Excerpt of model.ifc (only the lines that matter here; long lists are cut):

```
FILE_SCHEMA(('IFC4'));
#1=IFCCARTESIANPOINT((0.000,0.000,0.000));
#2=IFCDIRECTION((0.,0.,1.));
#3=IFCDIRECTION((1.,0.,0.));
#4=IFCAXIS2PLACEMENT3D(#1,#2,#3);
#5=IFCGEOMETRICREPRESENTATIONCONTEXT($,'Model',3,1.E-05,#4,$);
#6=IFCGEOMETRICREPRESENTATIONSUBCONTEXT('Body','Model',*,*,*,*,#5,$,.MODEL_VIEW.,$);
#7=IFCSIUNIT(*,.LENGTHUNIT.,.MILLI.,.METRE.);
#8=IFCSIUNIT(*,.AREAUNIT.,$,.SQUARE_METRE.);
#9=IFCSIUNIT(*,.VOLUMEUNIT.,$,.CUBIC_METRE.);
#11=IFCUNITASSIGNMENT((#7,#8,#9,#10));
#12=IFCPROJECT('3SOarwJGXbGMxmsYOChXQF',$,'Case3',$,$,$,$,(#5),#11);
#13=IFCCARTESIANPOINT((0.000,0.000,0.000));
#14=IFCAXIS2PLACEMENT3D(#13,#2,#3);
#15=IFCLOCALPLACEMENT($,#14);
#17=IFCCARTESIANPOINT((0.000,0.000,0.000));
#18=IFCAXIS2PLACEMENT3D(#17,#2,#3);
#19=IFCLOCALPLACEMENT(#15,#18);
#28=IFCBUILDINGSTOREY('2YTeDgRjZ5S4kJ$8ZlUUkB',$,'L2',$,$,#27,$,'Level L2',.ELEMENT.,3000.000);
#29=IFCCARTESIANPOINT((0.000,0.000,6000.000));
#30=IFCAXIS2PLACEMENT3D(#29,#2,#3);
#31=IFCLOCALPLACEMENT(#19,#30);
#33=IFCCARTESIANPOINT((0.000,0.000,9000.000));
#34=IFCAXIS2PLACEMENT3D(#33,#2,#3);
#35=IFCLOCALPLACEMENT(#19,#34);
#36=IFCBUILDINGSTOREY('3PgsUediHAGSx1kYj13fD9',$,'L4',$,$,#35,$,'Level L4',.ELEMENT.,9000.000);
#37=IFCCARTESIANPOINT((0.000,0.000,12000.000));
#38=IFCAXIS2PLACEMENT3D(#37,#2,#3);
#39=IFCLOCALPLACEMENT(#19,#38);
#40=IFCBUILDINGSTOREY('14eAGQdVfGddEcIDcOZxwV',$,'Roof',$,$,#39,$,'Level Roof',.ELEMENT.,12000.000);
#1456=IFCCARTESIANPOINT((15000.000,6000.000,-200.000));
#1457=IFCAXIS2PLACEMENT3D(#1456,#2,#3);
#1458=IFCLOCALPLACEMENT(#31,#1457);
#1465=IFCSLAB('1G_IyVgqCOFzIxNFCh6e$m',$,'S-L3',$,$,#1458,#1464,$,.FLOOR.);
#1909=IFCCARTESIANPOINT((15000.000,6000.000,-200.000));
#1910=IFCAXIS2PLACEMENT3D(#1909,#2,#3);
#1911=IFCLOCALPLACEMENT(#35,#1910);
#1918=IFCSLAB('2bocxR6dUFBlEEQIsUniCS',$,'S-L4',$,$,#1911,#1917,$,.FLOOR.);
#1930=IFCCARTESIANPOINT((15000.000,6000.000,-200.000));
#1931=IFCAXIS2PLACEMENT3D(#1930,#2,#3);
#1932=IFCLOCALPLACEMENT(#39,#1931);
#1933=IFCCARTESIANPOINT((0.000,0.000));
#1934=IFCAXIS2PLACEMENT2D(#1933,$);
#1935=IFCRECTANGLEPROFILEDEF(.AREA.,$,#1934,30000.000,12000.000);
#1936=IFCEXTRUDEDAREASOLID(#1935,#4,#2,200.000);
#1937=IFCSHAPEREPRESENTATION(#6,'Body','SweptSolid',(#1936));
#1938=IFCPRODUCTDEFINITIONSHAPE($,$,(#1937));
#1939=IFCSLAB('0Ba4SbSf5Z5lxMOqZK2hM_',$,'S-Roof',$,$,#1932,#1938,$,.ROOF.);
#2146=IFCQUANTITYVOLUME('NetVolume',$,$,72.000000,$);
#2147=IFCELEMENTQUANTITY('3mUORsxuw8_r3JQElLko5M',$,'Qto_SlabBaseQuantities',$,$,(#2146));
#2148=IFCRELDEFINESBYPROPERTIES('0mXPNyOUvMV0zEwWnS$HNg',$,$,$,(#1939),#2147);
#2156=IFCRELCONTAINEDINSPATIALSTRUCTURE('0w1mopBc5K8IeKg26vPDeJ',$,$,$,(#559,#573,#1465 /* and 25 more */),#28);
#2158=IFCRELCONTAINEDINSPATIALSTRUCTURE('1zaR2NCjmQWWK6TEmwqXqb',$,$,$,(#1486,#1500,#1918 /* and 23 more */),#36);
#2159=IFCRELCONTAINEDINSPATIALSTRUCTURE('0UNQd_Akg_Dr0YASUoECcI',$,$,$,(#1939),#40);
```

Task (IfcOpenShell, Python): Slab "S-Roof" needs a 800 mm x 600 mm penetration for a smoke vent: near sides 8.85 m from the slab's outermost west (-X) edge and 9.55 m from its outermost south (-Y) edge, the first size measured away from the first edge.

```python
import numpy as np
import ifcopenshell
import ifcopenshell.api.feature
import ifcopenshell.api.geometry
import ifcopenshell.api.pset
import ifcopenshell.api.root
import ifcopenshell.geom
import ifcopenshell.util.element
import ifcopenshell.util.placement
import ifcopenshell.util.representation
import ifcopenshell.util.shape
import ifcopenshell.util.unit

model = ifcopenshell.open("model.ifc")
unit_scale = ifcopenshell.util.unit.calculate_unit_scale(model)
volume_scale = ifcopenshell.util.unit.calculate_unit_scale(model, "VOLUMEUNIT")
settings = ifcopenshell.geom.settings()


def volume(element):
    """Net volume in cubic metres, openings subtracted."""
    shape = ifcopenshell.geom.create_shape(settings, element)
    return ifcopenshell.util.shape.get_volume(shape.geometry)


slab = model.by_id(1939)
before = volume(slab)

# Extent in the slab's own axes, in metres. The edges named are its -X and -Y sides.
slab_shape = ifcopenshell.geom.create_shape(settings, slab)
vertices = ifcopenshell.util.shape.get_vertices(slab_shape.geometry)
x_min, y_min, bottom = vertices.min(axis=0)
top = vertices[:, 2].max()

opening = ifcopenshell.api.root.create_entity(model, ifc_class="IfcOpeningElement", name="Smoke vent opening", predefined_type="OPENING")
context = ifcopenshell.util.representation.get_context(model, "Model", "Body", "MODEL_VIEW")
width, depth = 0.8, 0.6
outline = [(0.0, 0.0), (width, 0.0), (width, depth), (0.0, depth), (0.0, 0.0)]
# Overshoot both faces by 50 mm so the cut is clean.
shape = ifcopenshell.api.geometry.add_slab_representation(
    model, context=context, depth=top - bottom + 0.1, polyline=outline
)
ifcopenshell.api.geometry.assign_representation(model, product=opening, representation=shape)

matrix = ifcopenshell.util.placement.get_local_placement(slab.ObjectPlacement)
matrix[:, 3] = matrix @ np.append(np.array([x_min + 8.85, y_min + 9.55, bottom - 0.05]) / unit_scale, 1.0)
ifcopenshell.api.geometry.edit_object_placement(model, product=opening, matrix=matrix, is_si=False)
ifcopenshell.api.feature.add_feature(model, feature=opening, element=slab)

after = volume(slab)

# Update the slab's stored quantities.
qto = model.by_id(ifcopenshell.util.element.get_pset(slab, "Qto_SlabBaseQuantities", should_inherit=False)["id"])
ifcopenshell.api.pset.edit_qto(model, qto=qto, properties={"NetVolume": after / volume_scale})

print(f"slab volume {before:.3f} -> {after:.3f} m3")

model.write("model_v2.ifc")
```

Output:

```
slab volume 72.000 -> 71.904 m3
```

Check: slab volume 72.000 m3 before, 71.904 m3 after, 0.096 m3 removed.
